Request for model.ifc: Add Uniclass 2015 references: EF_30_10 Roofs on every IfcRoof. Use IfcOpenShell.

First a look at what the model holds.

```python
import ifcopenshell

model = ifcopenshell.open("model.ifc")
print(model.schema)
print("classifications:", [c.Name for c in model.by_type("IfcClassification")])
for ifc_class in ("IfcDoor", "IfcRoof", "IfcStair", "IfcWall", "IfcWindow"):
    print(ifc_class, len(model.by_type(ifc_class)))
```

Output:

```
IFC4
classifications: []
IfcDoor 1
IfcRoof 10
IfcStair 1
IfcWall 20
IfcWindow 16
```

```python
import ifcopenshell
import ifcopenshell.api.classification

model = ifcopenshell.open("model.ifc")

system = ifcopenshell.api.classification.add_classification(model, classification="Uniclass 2015")

codes = {
    "IfcRoof": ("EF_30_10", "Roofs"),
}
for ifc_class, (code, name) in codes.items():
    products = model.by_type(ifc_class)
    ifcopenshell.api.classification.add_reference(
        model, products=products, classification=system, identification=code, name=name
    )
    print(code, len(products))

model.write("model-out.ifc")
```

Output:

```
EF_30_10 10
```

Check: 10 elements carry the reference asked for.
